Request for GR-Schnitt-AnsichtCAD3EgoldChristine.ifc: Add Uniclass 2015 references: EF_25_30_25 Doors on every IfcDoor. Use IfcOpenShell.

First a look at what the model holds.

```python
import ifcopenshell

model = ifcopenshell.open("GR-Schnitt-AnsichtCAD3EgoldChristine.ifc")
print(model.schema)
print("classifications:", [c.Name for c in model.by_type("IfcClassification")])
for ifc_class in ("IfcDoor", "IfcRoof", "IfcStair", "IfcWall", "IfcWindow"):
    print(ifc_class, len(model.by_type(ifc_class)))
```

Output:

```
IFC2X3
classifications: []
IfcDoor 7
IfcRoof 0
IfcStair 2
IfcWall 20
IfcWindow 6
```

```python
import ifcopenshell
import ifcopenshell.api.classification

model = ifcopenshell.open("GR-Schnitt-AnsichtCAD3EgoldChristine.ifc")

# IFC2X3 requires Source and Edition and has no link from the project to the system.
system = model.create_entity("IfcClassification", Source="NBS", Edition="2015", Name="Uniclass 2015")

codes = {
    "IfcDoor": ("EF_25_30_25", "Doors"),
}
for ifc_class, (code, name) in codes.items():
    products = model.by_type(ifc_class)
    ifcopenshell.api.classification.add_reference(
        model, products=products, classification=system, identification=code, name=name
    )
    print(code, len(products))

model.write("GR-Schnitt-AnsichtCAD3EgoldChristine_edited.ifc")
```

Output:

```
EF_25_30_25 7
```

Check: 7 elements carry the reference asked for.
